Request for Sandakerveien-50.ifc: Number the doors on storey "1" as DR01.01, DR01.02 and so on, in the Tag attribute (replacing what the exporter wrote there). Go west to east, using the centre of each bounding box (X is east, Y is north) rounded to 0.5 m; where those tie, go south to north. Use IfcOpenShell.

First a look at what the model holds.

```python
import ifcopenshell
import ifcopenshell.util.element
import ifcopenshell.util.placement

model = ifcopenshell.open("Sandakerveien-50.ifc")
print(model.schema)
storey = next(s for s in model.by_type("IfcBuildingStorey") if s.Name == "1")
doors = [e for e in ifcopenshell.util.element.get_decomposition(storey) if e.is_a("IfcDoor")]
for e in sorted(doors, key=lambda e: e.id()):
    origin = ifcopenshell.util.placement.get_local_placement(e.ObjectPlacement)[:3, 3]
    print(e.id(), e.Tag, e.Name, origin.round(2) + 0.0, sep=" | ")
```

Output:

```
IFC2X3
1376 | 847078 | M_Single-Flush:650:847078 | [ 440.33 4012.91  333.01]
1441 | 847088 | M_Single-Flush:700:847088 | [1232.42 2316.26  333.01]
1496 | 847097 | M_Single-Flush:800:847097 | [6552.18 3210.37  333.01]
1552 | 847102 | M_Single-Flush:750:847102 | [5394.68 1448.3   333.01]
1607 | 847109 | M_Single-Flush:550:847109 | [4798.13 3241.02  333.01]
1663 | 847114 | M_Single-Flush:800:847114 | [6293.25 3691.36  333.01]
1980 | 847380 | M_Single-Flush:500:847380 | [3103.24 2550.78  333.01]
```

```python
import ifcopenshell
import ifcopenshell.geom
import ifcopenshell.util.element
import ifcopenshell.util.shape

model = ifcopenshell.open("Sandakerveien-50.ifc")
settings = ifcopenshell.geom.settings()
settings.set("use-world-coords", True)


def centre(element):
    shape = ifcopenshell.geom.create_shape(settings, element)
    return ifcopenshell.util.shape.get_bbox_centroid(shape.geometry)


storey = next(s for s in model.by_type("IfcBuildingStorey") if s.Name == "1")
doors = [e for e in ifcopenshell.util.element.get_decomposition(storey) if e.is_a("IfcDoor")]

# Insertion points can sit at a corner or the storey origin, so sort by the geometry (in metres).
centres = {e: centre(e) for e in doors}
doors.sort(key=lambda e: (round(centres[e][0] / 0.5), centres[e][1]))

for i, e in enumerate(doors, start=1):
    number = f"DR01.{i:02d}"
    e.Tag = number
    print(e.id(), number)

model.write("Sandakerveien-50-out.ifc")
```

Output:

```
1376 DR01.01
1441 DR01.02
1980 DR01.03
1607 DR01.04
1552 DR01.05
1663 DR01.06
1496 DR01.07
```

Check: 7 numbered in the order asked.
